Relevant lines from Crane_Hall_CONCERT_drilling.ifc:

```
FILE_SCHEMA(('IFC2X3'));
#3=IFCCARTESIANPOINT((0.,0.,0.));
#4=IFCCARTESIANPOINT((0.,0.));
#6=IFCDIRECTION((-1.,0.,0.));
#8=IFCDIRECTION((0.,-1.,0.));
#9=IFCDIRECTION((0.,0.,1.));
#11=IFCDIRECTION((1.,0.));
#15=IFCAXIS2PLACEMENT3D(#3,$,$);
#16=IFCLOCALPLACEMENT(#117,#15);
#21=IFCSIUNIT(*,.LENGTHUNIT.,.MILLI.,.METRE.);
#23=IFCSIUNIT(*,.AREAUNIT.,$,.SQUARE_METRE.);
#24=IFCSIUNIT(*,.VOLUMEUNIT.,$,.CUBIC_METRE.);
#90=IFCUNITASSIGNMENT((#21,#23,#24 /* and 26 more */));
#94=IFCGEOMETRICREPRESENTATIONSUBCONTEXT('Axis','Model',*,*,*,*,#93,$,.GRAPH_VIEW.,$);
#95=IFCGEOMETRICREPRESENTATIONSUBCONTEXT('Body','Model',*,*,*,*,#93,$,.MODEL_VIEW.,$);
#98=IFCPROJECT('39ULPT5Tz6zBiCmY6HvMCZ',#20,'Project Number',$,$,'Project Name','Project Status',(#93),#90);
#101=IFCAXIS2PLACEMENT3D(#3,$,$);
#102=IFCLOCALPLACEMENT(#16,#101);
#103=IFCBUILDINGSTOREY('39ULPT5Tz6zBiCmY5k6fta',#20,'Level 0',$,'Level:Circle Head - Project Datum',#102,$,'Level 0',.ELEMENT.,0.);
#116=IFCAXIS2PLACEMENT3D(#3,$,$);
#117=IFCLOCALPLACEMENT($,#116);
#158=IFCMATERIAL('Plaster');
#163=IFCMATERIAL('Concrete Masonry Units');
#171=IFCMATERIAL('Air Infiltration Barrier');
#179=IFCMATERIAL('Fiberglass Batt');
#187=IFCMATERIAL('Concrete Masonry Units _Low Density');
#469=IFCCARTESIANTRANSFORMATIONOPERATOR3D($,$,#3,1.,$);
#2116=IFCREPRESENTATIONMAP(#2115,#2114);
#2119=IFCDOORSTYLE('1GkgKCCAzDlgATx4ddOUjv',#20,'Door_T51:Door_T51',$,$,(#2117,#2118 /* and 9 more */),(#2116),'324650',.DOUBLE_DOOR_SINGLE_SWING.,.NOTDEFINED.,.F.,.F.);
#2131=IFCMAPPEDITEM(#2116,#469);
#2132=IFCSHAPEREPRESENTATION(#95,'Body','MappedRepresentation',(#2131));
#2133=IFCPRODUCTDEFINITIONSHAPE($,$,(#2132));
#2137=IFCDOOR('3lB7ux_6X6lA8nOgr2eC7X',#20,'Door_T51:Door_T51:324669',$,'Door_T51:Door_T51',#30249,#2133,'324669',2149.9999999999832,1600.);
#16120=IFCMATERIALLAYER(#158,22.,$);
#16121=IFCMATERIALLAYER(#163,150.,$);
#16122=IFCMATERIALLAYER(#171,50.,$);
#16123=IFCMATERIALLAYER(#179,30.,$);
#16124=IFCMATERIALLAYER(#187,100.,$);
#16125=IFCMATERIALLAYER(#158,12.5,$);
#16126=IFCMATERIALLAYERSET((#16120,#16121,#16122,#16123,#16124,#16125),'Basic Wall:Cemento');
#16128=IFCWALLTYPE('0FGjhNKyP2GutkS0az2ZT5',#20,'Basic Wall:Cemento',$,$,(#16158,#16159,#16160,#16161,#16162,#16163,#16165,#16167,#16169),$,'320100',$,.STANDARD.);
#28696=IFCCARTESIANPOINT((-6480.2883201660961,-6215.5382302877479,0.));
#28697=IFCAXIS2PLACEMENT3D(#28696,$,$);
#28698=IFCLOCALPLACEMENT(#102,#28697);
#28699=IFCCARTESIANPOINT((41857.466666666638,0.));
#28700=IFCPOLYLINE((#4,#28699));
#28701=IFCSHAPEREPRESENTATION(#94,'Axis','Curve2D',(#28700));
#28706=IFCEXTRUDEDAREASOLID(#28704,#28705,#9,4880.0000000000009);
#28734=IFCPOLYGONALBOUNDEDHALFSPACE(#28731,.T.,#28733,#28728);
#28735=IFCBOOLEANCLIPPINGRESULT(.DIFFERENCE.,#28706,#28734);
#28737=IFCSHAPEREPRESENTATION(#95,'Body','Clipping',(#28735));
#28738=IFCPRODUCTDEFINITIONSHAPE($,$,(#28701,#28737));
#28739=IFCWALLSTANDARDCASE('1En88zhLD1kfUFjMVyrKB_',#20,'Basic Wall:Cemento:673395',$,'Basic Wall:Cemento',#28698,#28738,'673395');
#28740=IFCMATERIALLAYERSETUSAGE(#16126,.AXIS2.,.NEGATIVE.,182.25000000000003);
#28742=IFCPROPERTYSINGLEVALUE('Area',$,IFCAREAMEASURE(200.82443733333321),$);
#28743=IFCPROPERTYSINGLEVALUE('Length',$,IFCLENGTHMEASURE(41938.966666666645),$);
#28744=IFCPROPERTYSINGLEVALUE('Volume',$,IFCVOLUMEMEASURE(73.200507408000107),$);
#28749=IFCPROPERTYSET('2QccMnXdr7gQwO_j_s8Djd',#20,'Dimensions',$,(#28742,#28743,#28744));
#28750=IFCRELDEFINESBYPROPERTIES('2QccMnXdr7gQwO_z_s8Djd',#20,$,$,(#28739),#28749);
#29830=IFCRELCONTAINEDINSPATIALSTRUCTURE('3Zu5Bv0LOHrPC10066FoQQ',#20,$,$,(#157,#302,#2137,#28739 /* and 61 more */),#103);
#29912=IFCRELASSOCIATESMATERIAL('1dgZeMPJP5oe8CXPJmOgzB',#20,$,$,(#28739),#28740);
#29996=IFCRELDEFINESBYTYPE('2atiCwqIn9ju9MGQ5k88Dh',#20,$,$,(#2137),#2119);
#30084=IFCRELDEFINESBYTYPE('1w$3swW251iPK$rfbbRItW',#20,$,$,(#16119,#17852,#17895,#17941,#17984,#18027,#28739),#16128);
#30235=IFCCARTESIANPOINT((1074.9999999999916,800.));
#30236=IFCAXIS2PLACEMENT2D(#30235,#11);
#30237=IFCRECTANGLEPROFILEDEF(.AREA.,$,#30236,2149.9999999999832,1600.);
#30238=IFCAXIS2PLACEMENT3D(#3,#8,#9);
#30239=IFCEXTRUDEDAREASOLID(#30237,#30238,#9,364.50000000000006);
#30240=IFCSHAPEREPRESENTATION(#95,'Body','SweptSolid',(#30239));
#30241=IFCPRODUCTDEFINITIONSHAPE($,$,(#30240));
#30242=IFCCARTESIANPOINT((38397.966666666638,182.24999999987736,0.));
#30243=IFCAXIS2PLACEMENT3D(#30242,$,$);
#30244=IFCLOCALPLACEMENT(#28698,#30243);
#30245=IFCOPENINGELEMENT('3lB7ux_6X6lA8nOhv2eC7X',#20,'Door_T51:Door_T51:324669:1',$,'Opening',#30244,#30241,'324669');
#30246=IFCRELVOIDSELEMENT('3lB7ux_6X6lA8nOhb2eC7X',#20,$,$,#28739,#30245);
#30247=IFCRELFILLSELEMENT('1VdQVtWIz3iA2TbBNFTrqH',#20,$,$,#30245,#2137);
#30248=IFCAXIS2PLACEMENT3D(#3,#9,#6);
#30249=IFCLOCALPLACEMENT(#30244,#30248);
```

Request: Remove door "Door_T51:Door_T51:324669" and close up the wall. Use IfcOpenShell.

```python
import ifcopenshell
import ifcopenshell.api.feature
import ifcopenshell.api.pset
import ifcopenshell.api.root
import ifcopenshell.geom
import ifcopenshell.util.element
import ifcopenshell.util.shape
import ifcopenshell.util.unit

model = ifcopenshell.open("Crane_Hall_CONCERT_drilling.ifc")
area_scale = ifcopenshell.util.unit.calculate_unit_scale(model, "AREAUNIT")
volume_scale = ifcopenshell.util.unit.calculate_unit_scale(model, "VOLUMEUNIT")
settings = ifcopenshell.geom.settings()


def volume(element):
    """Net volume in cubic metres, openings subtracted."""
    shape = ifcopenshell.geom.create_shape(settings, element)
    return ifcopenshell.util.shape.get_volume(shape.geometry)


door = model.by_id(2137)
opening = door.FillsVoids[0].RelatingOpeningElement
wall = opening.VoidsElements[0].RelatingBuildingElement
before = volume(wall)

ifcopenshell.api.root.remove_product(model, product=door)
ifcopenshell.api.feature.remove_feature(model, feature=opening)

after = volume(wall)
thickness = 0.3645  # wall thickness in metres

# Update the wall's stored quantities.
pset = model.by_id(ifcopenshell.util.element.get_pset(wall, "Dimensions", should_inherit=False)["id"])
ifcopenshell.api.pset.edit_pset(model, pset=pset, properties={
    "Area": model.create_entity("IfcAreaMeasure", after / thickness / area_scale),
    "Volume": model.create_entity("IfcVolumeMeasure", after / volume_scale),
})

print(f"wall volume {before:.3f} -> {after:.3f} m3")

model.write("Crane_Hall_CONCERT_drilling_updated.ifc")
```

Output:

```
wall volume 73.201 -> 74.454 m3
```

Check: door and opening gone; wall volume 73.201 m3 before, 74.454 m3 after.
